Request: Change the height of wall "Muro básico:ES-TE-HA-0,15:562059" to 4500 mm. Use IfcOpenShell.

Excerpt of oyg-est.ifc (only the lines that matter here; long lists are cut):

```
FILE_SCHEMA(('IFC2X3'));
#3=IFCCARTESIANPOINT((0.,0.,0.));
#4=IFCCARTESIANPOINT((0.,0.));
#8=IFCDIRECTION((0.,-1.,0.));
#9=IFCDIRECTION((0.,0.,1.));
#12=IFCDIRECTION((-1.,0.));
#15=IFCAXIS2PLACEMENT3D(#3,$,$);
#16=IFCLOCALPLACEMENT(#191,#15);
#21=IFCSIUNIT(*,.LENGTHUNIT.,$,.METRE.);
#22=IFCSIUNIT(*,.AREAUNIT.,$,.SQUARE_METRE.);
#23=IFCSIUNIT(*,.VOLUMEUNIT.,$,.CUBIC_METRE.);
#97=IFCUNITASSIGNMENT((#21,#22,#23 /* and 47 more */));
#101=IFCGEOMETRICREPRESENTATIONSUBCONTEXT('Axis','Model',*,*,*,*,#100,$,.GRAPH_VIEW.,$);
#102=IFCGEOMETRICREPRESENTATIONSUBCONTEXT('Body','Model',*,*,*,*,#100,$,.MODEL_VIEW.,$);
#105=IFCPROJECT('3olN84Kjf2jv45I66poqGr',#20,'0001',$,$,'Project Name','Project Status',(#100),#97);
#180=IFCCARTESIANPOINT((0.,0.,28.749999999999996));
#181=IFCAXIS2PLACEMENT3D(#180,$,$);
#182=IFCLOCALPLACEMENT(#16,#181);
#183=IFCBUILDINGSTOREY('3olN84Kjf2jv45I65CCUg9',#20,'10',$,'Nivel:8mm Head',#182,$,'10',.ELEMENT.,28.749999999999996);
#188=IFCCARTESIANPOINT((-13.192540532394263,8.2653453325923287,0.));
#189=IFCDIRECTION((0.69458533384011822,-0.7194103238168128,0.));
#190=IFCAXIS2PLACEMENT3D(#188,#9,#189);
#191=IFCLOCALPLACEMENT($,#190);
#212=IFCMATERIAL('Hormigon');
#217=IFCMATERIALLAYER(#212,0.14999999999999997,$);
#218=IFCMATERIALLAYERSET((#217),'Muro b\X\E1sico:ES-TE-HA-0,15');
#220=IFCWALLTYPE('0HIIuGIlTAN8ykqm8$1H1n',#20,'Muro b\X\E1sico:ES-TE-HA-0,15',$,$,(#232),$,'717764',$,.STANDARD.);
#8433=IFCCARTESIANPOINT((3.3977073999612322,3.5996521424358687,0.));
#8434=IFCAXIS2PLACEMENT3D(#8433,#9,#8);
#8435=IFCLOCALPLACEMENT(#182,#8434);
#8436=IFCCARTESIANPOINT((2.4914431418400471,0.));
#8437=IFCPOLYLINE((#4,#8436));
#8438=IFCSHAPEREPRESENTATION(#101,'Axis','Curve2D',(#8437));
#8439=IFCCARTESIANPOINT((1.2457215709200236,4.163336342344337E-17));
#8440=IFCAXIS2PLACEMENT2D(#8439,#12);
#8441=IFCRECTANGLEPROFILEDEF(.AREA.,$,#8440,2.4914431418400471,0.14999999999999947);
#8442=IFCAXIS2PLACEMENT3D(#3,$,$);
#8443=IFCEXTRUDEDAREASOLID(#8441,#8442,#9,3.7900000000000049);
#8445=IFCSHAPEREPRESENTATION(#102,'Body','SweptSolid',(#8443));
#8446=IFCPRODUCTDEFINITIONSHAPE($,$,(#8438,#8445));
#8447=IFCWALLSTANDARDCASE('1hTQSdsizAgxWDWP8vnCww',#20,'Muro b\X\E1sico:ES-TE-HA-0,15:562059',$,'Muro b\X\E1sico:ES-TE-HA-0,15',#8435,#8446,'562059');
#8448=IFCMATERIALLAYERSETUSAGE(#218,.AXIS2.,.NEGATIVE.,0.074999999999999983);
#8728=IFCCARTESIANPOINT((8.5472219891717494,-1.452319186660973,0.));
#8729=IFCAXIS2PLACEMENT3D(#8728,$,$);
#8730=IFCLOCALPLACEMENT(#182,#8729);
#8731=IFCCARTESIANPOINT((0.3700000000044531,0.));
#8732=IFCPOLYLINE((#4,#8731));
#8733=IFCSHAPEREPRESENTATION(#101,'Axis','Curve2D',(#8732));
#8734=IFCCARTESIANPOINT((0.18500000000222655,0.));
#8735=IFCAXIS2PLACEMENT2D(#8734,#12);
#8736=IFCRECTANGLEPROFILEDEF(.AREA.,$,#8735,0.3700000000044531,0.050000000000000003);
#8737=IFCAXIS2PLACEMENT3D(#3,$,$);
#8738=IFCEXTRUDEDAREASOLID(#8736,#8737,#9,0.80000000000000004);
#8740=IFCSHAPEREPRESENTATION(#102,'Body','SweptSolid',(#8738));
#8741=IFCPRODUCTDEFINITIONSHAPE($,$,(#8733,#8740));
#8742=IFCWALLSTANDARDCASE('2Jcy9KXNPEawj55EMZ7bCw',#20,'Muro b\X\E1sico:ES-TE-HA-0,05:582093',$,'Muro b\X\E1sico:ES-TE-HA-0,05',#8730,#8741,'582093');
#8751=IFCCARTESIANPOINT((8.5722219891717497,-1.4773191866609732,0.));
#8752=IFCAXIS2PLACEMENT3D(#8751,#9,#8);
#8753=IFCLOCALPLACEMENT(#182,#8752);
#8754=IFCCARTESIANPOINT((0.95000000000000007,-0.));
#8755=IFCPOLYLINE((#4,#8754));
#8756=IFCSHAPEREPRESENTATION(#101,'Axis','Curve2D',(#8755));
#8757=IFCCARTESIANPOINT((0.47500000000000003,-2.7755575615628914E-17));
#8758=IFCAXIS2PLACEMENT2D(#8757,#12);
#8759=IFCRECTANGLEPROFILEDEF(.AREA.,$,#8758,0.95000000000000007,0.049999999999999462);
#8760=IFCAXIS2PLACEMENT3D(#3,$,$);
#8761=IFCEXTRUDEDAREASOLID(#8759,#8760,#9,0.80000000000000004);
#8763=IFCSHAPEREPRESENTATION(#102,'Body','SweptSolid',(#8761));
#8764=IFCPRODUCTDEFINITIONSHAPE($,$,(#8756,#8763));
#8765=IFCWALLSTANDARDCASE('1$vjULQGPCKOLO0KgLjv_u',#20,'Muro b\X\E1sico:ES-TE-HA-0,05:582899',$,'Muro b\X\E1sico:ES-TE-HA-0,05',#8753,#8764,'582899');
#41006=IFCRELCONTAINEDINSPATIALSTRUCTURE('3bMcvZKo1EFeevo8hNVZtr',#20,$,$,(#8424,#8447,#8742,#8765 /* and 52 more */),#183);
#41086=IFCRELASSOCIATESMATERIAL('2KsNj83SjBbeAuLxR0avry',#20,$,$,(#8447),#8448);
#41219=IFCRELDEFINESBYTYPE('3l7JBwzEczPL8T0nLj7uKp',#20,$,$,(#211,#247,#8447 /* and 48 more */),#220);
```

```python
import ifcopenshell
import ifcopenshell.geom
import ifcopenshell.util.representation
import ifcopenshell.util.shape

model = ifcopenshell.open("oyg-est.ifc")
settings = ifcopenshell.geom.settings()


def volume(element):
    """Net volume in cubic metres, openings subtracted."""
    shape = ifcopenshell.geom.create_shape(settings, element)
    return ifcopenshell.util.shape.get_volume(shape.geometry)


wall = model.by_guid("1hTQSdsizAgxWDWP8vnCww")
before = volume(wall)

body = ifcopenshell.util.representation.get_representation(wall, "Model", "Body")
solid = body.Items[0]
old_height = solid.Depth
solid.Depth = 4.5
after = volume(wall)

print(f"height {old_height:g} -> {solid.Depth:g}, volume {before:.3f} -> {after:.3f} m3")

model.write("oyg-est_v2.ifc")
```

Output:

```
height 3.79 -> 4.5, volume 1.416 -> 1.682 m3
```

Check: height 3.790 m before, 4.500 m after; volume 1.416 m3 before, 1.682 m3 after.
